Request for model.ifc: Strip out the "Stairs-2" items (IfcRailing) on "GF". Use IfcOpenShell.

First a look at what the model holds.

```python
import ifcopenshell
import ifcopenshell.util.element

model = ifcopenshell.open("model.ifc")
print(model.schema)
storey = next(s for s in model.by_type("IfcBuildingStorey") if s.Name == "GF")
railings = [e for e in ifcopenshell.util.element.get_decomposition(storey) if e.is_a("IfcRailing")]
seen = {}
for e in railings:
    element_type = ifcopenshell.util.element.get_type(e)
    name = element_type.Name if element_type not in (None, e) else None
    seen[name] = seen.get(name, 0) + 1
for name, count in sorted(seen.items(), key=str):
    print(count, "x", name)
```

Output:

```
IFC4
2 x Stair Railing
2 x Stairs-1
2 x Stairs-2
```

```python
import ifcopenshell
import ifcopenshell.api.root
import ifcopenshell.util.element

model = ifcopenshell.open("model.ifc")

storey = next(s for s in model.by_type("IfcBuildingStorey") if s.Name == "GF")
railings = [e for e in ifcopenshell.util.element.get_decomposition(storey) if e.is_a("IfcRailing")]
targets = [e for e in railings if (t := ifcopenshell.util.element.get_type(e)) not in (None, e) and t.Name == "Stairs-2"]

for e in targets:
    ifcopenshell.api.root.remove_product(model, product=e)
print(len(targets), "removed")

model.write("model_v2.ifc")
```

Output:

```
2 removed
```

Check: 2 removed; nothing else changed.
